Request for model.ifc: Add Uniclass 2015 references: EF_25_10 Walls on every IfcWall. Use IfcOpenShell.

First a look at what the model holds.

```python
import ifcopenshell

model = ifcopenshell.open("model.ifc")
print(model.schema)
print("classifications:", [c.Name for c in model.by_type("IfcClassification")])
for ifc_class in ("IfcDoor", "IfcRoof", "IfcStair", "IfcWall", "IfcWindow"):
    print(ifc_class, len(model.by_type(ifc_class)))
```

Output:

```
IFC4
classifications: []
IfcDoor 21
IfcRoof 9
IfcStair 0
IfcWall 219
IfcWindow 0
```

```python
import ifcopenshell
import ifcopenshell.api.classification

model = ifcopenshell.open("model.ifc")

system = ifcopenshell.api.classification.add_classification(model, classification="Uniclass 2015")

codes = {
    "IfcWall": ("EF_25_10", "Walls"),
}
for ifc_class, (code, name) in codes.items():
    products = model.by_type(ifc_class)
    ifcopenshell.api.classification.add_reference(
        model, products=products, classification=system, identification=code, name=name
    )
    print(code, len(products))

model.write("model_rev.ifc")
```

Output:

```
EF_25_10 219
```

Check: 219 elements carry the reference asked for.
